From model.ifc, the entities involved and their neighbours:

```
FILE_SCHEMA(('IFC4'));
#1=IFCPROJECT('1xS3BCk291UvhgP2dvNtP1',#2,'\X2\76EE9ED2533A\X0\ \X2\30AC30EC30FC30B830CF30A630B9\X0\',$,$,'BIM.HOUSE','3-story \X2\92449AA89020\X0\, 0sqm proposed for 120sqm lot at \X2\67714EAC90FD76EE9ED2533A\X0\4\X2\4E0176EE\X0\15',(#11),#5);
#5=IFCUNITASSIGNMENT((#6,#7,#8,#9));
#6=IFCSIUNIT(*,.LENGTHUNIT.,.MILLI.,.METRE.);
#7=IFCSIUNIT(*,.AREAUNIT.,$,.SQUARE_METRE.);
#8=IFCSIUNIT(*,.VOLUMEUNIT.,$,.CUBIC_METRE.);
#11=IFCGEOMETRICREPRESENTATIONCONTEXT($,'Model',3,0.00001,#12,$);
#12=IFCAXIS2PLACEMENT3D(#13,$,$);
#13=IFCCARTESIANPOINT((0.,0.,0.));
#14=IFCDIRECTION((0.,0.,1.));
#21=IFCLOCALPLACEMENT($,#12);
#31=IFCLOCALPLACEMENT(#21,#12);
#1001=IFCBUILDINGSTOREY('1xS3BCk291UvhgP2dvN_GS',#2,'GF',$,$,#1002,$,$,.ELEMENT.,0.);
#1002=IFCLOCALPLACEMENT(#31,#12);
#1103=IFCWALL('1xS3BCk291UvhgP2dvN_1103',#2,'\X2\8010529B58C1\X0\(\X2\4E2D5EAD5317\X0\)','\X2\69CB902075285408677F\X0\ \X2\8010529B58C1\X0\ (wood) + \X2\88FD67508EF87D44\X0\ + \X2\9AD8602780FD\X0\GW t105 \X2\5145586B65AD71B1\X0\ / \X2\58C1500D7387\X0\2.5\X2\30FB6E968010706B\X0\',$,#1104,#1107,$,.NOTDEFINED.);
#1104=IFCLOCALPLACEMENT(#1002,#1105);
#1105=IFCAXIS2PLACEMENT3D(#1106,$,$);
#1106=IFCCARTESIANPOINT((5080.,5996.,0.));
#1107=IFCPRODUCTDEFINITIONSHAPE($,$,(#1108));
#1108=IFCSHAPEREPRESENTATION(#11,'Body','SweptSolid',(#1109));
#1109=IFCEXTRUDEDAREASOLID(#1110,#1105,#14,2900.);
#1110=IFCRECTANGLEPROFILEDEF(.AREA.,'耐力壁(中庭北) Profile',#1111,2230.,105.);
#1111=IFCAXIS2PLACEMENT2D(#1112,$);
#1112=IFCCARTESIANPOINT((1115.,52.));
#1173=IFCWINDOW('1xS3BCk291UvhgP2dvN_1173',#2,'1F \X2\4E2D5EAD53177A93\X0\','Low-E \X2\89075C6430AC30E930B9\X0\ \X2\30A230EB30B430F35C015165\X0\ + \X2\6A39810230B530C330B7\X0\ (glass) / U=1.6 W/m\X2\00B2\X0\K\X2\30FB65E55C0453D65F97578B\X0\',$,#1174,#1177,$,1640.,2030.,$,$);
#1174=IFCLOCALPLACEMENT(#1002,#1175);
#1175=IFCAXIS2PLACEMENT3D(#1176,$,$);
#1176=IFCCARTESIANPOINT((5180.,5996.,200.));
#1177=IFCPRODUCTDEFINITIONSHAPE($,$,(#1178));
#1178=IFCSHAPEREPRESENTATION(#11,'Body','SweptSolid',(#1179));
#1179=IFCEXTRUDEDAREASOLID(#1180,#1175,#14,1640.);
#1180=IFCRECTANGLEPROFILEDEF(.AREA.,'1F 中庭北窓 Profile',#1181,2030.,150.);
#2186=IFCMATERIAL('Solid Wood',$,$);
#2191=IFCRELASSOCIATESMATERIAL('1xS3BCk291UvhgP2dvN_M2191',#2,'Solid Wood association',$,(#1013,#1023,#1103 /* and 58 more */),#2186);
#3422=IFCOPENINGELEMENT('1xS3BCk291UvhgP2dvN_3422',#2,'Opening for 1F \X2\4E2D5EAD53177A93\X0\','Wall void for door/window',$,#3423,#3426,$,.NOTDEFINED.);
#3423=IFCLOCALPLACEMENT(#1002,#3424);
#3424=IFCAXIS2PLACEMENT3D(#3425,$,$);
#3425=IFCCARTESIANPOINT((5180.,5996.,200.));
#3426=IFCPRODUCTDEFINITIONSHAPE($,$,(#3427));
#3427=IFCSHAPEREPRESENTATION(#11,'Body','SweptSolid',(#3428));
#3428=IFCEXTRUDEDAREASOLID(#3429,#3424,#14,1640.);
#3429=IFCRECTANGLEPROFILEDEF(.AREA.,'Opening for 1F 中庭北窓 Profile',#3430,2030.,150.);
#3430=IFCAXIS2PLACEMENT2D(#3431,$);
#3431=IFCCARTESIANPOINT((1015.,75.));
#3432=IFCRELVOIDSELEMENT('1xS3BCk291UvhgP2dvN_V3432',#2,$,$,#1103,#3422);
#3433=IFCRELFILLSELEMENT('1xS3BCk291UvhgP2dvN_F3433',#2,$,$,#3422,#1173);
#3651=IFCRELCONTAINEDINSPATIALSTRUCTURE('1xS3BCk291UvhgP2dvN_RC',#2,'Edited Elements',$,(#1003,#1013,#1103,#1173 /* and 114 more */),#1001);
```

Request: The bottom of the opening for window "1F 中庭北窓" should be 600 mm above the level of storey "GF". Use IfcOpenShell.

```python
import numpy as np
import ifcopenshell
import ifcopenshell.api.geometry
import ifcopenshell.geom
import ifcopenshell.util.element
import ifcopenshell.util.placement
import ifcopenshell.util.shape
import ifcopenshell.util.unit

model = ifcopenshell.open("model.ifc")
unit_scale = ifcopenshell.util.unit.calculate_unit_scale(model)

window = model.by_guid("1xS3BCk291UvhgP2dvN_1173")
opening = window.FillsVoids[0].RelatingOpeningElement
storey = ifcopenshell.util.element.get_container(window, ifc_class="IfcBuildingStorey")
level = ifcopenshell.util.placement.get_local_placement(storey.ObjectPlacement)[2, 3]

# The opening's origin need not be at the sill, so measure its lowest point.
shape = ifcopenshell.geom.create_shape(ifcopenshell.geom.settings(), opening)
bottom = ifcopenshell.util.shape.get_shape_bottom_elevation(shape, shape.geometry) / unit_scale
dz = level + 600.0 - bottom

shift = np.array([0.0, 0.0, dz])
# The window is not placed relative to its opening, so move both.
for product in (opening, window):
    matrix = ifcopenshell.util.placement.get_local_placement(product.ObjectPlacement)
    matrix[:3, 3] += shift
    ifcopenshell.api.geometry.edit_object_placement(model, product=product, matrix=matrix, is_si=False)

print(f"moved by {dz * unit_scale:+.3f} m")

model.write("model_rev.ifc")
```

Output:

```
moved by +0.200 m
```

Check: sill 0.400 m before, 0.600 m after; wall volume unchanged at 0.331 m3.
